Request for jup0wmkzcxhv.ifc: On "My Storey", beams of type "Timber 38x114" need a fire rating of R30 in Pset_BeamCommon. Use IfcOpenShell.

First a look at what the model holds.

```python
import ifcopenshell
import ifcopenshell.util.element

model = ifcopenshell.open("jup0wmkzcxhv.ifc")
print(model.schema)
storey = next(s for s in model.by_type("IfcBuildingStorey") if s.Name == "My Storey")
beams = [e for e in ifcopenshell.util.element.get_decomposition(storey) if e.is_a("IfcBeam")]
seen = {}
for e in beams:
    element_type = ifcopenshell.util.element.get_type(e)
    key = (element_type.Name if element_type != e and element_type else None, ifcopenshell.util.element.get_pset(e, "Pset_BeamCommon", "FireRating"))
    seen[key] = seen.get(key, 0) + 1
for (name, value), count in sorted(seen.items(), key=str):
    print(count, "x", name, "|", value)
```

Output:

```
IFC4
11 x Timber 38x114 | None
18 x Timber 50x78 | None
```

```python
import ifcopenshell
import ifcopenshell.api.pset
import ifcopenshell.util.element

model = ifcopenshell.open("jup0wmkzcxhv.ifc")

storey = next(s for s in model.by_type("IfcBuildingStorey") if s.Name == "My Storey")
beams = [e for e in ifcopenshell.util.element.get_decomposition(storey) if e.is_a("IfcBeam")]

count = 0
for e in beams:
    element_type = ifcopenshell.util.element.get_type(e)
    if element_type in (None, e) or element_type.Name != "Timber 38x114":
        continue
    # add_pset returns the element's existing set when there is one.
    pset = ifcopenshell.api.pset.add_pset(model, product=e, name="Pset_BeamCommon")
    ifcopenshell.api.pset.edit_pset(model, pset=pset, properties={"FireRating": "R30"})
    count += 1

print(count, "beams updated")

model.write("jup0wmkzcxhv_rev.ifc")
```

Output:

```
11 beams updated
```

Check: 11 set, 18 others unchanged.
